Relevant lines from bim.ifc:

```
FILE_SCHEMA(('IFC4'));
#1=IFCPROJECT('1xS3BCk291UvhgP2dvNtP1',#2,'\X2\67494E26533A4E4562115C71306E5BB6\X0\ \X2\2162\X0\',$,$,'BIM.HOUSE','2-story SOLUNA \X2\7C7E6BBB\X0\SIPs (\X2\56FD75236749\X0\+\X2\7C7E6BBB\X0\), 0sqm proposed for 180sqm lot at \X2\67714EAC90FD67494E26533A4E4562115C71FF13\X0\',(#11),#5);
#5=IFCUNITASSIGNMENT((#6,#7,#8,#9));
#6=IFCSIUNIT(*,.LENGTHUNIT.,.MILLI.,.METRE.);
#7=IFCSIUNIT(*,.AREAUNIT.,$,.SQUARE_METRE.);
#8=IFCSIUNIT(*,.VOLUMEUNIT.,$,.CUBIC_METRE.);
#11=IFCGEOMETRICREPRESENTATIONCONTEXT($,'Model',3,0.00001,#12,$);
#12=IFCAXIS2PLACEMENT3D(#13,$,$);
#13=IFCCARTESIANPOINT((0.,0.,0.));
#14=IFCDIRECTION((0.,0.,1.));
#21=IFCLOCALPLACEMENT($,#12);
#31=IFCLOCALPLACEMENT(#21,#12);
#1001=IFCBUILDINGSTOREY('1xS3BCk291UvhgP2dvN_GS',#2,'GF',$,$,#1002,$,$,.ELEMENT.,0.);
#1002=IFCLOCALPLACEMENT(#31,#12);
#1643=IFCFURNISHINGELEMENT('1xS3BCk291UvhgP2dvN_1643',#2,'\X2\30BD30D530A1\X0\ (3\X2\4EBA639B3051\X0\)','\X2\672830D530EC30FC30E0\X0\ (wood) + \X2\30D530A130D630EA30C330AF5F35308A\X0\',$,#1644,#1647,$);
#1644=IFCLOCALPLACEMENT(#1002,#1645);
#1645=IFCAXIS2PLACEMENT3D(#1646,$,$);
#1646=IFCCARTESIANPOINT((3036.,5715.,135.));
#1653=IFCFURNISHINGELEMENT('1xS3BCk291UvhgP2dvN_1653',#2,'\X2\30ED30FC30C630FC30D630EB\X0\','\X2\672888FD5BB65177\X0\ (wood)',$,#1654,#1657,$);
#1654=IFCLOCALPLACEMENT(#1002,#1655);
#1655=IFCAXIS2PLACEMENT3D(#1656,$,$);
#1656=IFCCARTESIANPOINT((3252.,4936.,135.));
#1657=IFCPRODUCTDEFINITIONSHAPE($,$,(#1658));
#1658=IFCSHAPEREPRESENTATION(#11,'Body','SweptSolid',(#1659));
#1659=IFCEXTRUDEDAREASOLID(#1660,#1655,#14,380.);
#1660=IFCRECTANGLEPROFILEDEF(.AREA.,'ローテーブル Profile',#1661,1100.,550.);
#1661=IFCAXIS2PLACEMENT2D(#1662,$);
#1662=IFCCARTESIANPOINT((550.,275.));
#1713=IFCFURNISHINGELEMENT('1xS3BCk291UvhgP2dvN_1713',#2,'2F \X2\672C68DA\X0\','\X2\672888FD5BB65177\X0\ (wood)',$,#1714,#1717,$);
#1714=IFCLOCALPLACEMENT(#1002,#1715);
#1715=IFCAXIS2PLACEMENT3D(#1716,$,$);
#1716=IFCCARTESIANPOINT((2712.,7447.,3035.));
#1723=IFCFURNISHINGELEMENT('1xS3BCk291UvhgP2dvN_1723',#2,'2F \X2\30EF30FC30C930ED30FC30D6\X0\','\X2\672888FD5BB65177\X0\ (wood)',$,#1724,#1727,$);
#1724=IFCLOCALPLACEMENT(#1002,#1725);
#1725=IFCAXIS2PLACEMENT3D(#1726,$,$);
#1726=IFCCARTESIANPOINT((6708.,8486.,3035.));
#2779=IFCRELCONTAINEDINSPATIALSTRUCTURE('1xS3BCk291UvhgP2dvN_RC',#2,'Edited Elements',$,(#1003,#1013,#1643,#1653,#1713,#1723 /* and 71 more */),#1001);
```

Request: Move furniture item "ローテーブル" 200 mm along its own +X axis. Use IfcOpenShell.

```python
import ifcopenshell
import ifcopenshell.api.geometry
import ifcopenshell.util.placement
import ifcopenshell.util.unit

model = ifcopenshell.open("bim.ifc")
unit_scale = ifcopenshell.util.unit.calculate_unit_scale(model)

item = model.by_guid("1xS3BCk291UvhgP2dvN_1653")
matrix = ifcopenshell.util.placement.get_local_placement(item.ObjectPlacement)
matrix[:3, 3] += matrix[:3, 0] * 0.2 / unit_scale
ifcopenshell.api.geometry.edit_object_placement(model, product=item, matrix=matrix, is_si=False)

print(ifcopenshell.util.placement.get_local_placement(item.ObjectPlacement).round(3) + 0.0)

model.write("bim_v2.ifc")
```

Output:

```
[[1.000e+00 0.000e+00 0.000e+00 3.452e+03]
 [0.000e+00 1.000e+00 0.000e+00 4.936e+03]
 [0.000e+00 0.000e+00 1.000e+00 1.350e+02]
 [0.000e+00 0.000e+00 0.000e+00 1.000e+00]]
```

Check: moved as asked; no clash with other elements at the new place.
